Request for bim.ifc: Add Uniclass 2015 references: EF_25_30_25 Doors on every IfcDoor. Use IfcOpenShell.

First a look at what the model holds.

```python
import ifcopenshell

model = ifcopenshell.open("bim.ifc")
print(model.schema)
print("classifications:", [c.Name for c in model.by_type("IfcClassification")])
for ifc_class in ("IfcDoor", "IfcRoof", "IfcStair", "IfcWall", "IfcWindow"):
    print(ifc_class, len(model.by_type(ifc_class)))
```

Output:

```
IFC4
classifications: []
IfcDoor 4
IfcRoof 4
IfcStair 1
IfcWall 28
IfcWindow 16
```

```python
import ifcopenshell
import ifcopenshell.api.classification

model = ifcopenshell.open("bim.ifc")

system = ifcopenshell.api.classification.add_classification(model, classification="Uniclass 2015")

codes = {
    "IfcDoor": ("EF_25_30_25", "Doors"),
}
for ifc_class, (code, name) in codes.items():
    products = model.by_type(ifc_class)
    ifcopenshell.api.classification.add_reference(
        model, products=products, classification=system, identification=code, name=name
    )
    print(code, len(products))

model.write("bim_rev.ifc")
```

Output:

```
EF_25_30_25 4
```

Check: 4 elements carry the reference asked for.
